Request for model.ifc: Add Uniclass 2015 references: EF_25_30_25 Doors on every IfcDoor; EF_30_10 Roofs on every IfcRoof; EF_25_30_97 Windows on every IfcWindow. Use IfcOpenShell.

First a look at what the model holds.

```python
import ifcopenshell

model = ifcopenshell.open("model.ifc")
print(model.schema)
print("classifications:", [c.Name for c in model.by_type("IfcClassification")])
for ifc_class in ("IfcDoor", "IfcRoof", "IfcStair", "IfcWall", "IfcWindow"):
    print(ifc_class, len(model.by_type(ifc_class)))
```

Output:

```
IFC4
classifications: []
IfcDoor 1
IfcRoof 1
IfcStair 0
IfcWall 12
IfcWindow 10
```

```python
import ifcopenshell
import ifcopenshell.api.classification

model = ifcopenshell.open("model.ifc")

system = ifcopenshell.api.classification.add_classification(model, classification="Uniclass 2015")

codes = {
    "IfcDoor": ("EF_25_30_25", "Doors"),
    "IfcRoof": ("EF_30_10", "Roofs"),
    "IfcWindow": ("EF_25_30_97", "Windows"),
}
for ifc_class, (code, name) in codes.items():
    products = model.by_type(ifc_class)
    ifcopenshell.api.classification.add_reference(
        model, products=products, classification=system, identification=code, name=name
    )
    print(code, len(products))

model.write("model_edited.ifc")
```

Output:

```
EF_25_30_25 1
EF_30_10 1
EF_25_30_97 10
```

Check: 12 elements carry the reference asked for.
